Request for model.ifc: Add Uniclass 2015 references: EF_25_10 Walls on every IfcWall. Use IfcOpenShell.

First a look at what the model holds.

```python
import ifcopenshell

model = ifcopenshell.open("model.ifc")
print(model.schema)
print("classifications:", [c.Name for c in model.by_type("IfcClassification")])
for ifc_class in ("IfcDoor", "IfcRoof", "IfcStair", "IfcWall", "IfcWindow"):
    print(ifc_class, len(model.by_type(ifc_class)))
```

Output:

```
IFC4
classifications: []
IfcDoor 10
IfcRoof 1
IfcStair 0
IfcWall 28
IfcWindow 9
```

```python
import ifcopenshell
import ifcopenshell.api.classification

model = ifcopenshell.open("model.ifc")

system = ifcopenshell.api.classification.add_classification(model, classification="Uniclass 2015")

codes = {
    "IfcWall": ("EF_25_10", "Walls"),
}
for ifc_class, (code, name) in codes.items():
    products = model.by_type(ifc_class)
    ifcopenshell.api.classification.add_reference(
        model, products=products, classification=system, identification=code, name=name
    )
    print(code, len(products))

model.write("model_edited.ifc")
```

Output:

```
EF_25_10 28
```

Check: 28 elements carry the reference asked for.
